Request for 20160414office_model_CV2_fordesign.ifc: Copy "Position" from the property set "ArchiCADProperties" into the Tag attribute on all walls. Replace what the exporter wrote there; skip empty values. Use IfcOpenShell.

First a look at what the model holds.

```python
import ifcopenshell
import ifcopenshell.util.element

model = ifcopenshell.open("20160414office_model_CV2_fordesign.ifc")
print(model.schema)
walls = model.by_type("IfcWall")
print(len(walls), "walls")
for e in walls[:8]:
    source = ifcopenshell.util.element.get_pset(e, "ArchiCADProperties", "Position")
    target = e.Tag
    print(e.id(), repr(source), repr(target), sep=" | ")
```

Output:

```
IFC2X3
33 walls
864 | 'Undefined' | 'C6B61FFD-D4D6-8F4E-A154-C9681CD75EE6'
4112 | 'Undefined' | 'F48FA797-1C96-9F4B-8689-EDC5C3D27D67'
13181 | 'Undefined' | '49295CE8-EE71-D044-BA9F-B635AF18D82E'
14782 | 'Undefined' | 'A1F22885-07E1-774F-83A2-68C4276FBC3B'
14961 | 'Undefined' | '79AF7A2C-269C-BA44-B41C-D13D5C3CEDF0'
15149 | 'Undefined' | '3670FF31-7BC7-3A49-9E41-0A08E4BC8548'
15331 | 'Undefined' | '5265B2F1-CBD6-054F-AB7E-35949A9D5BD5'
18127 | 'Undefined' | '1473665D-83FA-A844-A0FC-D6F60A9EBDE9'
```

```python
import ifcopenshell
import ifcopenshell.util.element

model = ifcopenshell.open("20160414office_model_CV2_fordesign.ifc")

count = 0
for e in model.by_type("IfcWall"):
    value = ifcopenshell.util.element.get_pset(e, "ArchiCADProperties", "Position")
    current = e.Tag
    if not value or not value.strip() or current == value:
        continue
    e.Tag = value
    count += 1

print(count, "walls updated")

model.write("20160414office_model_CV2_fordesign_edited.ifc")
```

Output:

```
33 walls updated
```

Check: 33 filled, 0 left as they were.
